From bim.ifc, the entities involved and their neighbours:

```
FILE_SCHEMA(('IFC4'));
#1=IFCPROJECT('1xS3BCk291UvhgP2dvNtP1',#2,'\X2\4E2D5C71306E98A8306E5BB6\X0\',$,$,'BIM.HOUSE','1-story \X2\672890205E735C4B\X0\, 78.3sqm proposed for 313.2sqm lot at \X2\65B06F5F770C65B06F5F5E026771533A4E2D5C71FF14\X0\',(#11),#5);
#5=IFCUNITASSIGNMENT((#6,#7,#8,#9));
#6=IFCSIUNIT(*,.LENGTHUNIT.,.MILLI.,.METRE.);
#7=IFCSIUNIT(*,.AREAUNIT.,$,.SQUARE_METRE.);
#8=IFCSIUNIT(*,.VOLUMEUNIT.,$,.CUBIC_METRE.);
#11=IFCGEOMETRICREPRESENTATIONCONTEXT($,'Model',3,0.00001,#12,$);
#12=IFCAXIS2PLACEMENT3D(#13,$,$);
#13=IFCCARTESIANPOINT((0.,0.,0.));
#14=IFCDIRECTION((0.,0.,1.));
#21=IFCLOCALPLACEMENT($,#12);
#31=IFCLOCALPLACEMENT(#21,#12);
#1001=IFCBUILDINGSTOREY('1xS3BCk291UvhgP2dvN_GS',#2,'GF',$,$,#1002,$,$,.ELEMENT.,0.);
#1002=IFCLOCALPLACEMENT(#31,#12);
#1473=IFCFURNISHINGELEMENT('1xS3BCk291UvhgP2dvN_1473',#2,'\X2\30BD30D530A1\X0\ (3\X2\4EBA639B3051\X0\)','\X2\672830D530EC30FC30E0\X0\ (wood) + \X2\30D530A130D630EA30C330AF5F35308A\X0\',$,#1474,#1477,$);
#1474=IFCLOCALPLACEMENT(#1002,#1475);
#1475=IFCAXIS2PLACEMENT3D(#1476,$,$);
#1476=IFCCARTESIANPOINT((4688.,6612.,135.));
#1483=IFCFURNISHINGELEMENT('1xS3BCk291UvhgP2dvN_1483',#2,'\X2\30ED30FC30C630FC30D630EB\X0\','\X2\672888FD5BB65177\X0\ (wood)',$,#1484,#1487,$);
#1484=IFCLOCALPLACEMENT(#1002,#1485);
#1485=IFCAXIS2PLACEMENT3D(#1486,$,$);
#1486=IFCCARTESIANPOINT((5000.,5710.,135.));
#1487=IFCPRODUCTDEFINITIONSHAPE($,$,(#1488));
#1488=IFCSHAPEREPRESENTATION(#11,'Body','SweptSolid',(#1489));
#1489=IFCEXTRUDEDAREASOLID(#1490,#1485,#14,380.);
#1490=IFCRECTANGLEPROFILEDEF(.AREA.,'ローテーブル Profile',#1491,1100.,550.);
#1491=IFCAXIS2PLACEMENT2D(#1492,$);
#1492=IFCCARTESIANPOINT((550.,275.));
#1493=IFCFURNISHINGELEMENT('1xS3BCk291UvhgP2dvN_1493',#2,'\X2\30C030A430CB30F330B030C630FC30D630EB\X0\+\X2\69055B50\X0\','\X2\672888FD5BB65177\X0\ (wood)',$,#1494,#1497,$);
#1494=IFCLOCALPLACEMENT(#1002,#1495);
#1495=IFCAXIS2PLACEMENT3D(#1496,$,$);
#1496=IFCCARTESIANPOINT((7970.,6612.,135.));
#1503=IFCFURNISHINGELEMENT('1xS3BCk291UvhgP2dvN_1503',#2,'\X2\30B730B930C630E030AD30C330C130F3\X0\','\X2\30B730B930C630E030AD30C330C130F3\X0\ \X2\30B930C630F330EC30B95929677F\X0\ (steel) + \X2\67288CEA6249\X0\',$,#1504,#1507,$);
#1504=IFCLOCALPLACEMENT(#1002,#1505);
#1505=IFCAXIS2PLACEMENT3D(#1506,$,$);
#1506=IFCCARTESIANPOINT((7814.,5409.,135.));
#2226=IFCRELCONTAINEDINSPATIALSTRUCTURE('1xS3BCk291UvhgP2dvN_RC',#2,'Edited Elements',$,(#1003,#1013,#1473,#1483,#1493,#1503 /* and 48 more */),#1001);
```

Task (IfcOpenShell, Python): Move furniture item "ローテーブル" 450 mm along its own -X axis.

```python
import ifcopenshell
import ifcopenshell.api.geometry
import ifcopenshell.util.placement
import ifcopenshell.util.unit

model = ifcopenshell.open("bim.ifc")
unit_scale = ifcopenshell.util.unit.calculate_unit_scale(model)

item = model.by_guid("1xS3BCk291UvhgP2dvN_1483")
matrix = ifcopenshell.util.placement.get_local_placement(item.ObjectPlacement)
matrix[:3, 3] -= matrix[:3, 0] * 0.45 / unit_scale
ifcopenshell.api.geometry.edit_object_placement(model, product=item, matrix=matrix, is_si=False)

print(ifcopenshell.util.placement.get_local_placement(item.ObjectPlacement).round(3) + 0.0)

model.write("bim-out.ifc")
```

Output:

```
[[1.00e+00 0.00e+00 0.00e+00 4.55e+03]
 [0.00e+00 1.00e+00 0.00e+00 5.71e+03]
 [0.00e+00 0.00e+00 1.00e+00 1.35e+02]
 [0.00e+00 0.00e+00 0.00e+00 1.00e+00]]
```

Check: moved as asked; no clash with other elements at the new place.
